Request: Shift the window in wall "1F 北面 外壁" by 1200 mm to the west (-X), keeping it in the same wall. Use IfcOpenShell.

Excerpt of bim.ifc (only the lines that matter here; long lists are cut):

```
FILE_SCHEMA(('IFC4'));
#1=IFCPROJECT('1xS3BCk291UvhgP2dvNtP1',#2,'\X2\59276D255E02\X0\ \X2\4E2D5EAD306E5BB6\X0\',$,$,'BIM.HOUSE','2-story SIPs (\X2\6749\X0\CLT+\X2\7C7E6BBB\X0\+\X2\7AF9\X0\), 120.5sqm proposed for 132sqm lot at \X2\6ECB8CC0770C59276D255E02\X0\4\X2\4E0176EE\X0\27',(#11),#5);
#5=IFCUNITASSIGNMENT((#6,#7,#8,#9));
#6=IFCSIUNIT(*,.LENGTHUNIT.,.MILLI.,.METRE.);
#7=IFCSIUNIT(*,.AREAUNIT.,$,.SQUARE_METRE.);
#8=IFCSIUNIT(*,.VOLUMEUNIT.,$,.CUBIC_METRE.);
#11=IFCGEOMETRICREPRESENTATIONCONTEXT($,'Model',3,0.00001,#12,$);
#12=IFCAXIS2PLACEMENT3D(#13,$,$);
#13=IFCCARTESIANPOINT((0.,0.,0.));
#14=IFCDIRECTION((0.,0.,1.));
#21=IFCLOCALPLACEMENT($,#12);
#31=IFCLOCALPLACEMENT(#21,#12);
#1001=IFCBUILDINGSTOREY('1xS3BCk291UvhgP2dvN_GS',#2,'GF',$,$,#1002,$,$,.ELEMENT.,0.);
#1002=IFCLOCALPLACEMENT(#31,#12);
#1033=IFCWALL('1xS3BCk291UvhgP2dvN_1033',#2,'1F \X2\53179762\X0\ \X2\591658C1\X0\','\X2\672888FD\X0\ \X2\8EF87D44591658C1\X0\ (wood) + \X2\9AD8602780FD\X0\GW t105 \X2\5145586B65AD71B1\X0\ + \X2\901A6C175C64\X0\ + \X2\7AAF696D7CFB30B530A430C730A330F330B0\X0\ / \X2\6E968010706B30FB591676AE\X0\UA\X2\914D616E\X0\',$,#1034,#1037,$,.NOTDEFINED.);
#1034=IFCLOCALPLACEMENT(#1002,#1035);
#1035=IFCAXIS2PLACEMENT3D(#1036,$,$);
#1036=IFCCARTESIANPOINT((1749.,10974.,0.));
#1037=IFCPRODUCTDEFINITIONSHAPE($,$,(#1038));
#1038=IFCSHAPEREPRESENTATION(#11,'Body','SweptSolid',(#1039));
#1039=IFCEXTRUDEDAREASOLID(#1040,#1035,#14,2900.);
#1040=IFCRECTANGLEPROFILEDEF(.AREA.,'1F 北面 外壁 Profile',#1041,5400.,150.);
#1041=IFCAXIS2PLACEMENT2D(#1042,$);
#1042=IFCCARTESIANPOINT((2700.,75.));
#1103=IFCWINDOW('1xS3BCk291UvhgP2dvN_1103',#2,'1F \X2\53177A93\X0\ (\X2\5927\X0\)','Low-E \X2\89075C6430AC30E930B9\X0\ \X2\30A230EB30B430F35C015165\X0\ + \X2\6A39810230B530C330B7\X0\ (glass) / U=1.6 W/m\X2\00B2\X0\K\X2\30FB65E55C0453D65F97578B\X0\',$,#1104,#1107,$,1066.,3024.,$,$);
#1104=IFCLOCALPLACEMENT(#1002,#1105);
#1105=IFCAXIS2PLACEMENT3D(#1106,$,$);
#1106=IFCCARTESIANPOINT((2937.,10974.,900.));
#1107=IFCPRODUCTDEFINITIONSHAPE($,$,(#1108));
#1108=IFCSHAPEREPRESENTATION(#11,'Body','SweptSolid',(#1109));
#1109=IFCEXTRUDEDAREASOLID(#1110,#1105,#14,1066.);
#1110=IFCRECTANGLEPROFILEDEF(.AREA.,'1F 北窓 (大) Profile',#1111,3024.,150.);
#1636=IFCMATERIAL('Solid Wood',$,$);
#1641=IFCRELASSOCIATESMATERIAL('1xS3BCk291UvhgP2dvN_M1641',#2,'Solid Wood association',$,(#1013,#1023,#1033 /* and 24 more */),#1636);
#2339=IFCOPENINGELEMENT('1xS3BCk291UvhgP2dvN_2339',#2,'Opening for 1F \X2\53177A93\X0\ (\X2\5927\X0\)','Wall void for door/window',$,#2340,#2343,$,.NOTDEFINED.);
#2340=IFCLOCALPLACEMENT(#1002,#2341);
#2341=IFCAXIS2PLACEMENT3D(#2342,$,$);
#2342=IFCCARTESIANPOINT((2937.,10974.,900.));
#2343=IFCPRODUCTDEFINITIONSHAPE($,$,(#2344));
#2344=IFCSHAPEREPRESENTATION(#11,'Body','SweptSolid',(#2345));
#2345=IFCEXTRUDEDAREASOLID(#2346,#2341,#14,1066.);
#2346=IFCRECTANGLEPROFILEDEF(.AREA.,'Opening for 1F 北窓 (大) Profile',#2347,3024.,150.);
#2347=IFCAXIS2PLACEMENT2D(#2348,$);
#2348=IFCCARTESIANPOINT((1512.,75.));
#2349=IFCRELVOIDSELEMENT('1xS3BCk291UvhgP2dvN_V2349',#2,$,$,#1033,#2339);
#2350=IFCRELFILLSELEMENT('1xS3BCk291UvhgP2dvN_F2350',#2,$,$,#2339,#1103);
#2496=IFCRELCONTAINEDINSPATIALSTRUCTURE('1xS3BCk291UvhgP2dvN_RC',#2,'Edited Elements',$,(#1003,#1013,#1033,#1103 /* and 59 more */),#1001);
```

```python
import ifcopenshell
import ifcopenshell.api.geometry
import ifcopenshell.util.placement
import ifcopenshell.util.unit

model = ifcopenshell.open("bim.ifc")
unit_scale = ifcopenshell.util.unit.calculate_unit_scale(model)

window = model.by_guid("1xS3BCk291UvhgP2dvN_1103")
opening = window.FillsVoids[0].RelatingOpeningElement
wall = opening.VoidsElements[0].RelatingBuildingElement

wall_matrix = ifcopenshell.util.placement.get_local_placement(wall.ObjectPlacement)
shift = wall_matrix[:3, 0] * -1.2 / unit_scale
before = ifcopenshell.util.placement.get_local_placement(window.ObjectPlacement)[:3, 3].copy()

# The window is not placed relative to its opening, so move both.
for product in (opening, window):
    matrix = ifcopenshell.util.placement.get_local_placement(product.ObjectPlacement)
    matrix[:3, 3] += shift
    ifcopenshell.api.geometry.edit_object_placement(model, product=product, matrix=matrix, is_si=False)

after = ifcopenshell.util.placement.get_local_placement(window.ObjectPlacement)[:3, 3]
print("window moved by", (after - before).round(3) + 0.0)

model.write("bim_v2.ifc")
```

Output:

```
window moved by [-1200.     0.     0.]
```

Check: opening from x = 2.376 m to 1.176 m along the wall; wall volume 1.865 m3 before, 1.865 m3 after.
